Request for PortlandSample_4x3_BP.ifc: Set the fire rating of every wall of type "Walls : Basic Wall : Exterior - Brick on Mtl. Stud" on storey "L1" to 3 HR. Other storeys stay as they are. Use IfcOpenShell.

First a look at what the model holds.

```python
import ifcopenshell
import ifcopenshell.util.element

model = ifcopenshell.open("PortlandSample_4x3_BP.ifc")
print(model.schema)
storey = next(s for s in model.by_type("IfcBuildingStorey") if s.Name == "L1")
walls = [e for e in ifcopenshell.util.element.get_decomposition(storey) if e.is_a("IfcWall")]
seen = {}
for e in walls:
    element_type = ifcopenshell.util.element.get_type(e)
    key = (element_type.Name if element_type != e and element_type else None, ifcopenshell.util.element.get_pset(e, "Pset_WallCommon", "FireRating"))
    seen[key] = seen.get(key, 0) + 1
for (name, value), count in sorted(seen.items(), key=str):
    print(count, "x", name, "|", value)
```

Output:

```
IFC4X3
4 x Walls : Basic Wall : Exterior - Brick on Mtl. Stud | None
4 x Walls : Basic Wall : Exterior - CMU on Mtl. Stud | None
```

```python
import ifcopenshell
import ifcopenshell.api.pset
import ifcopenshell.util.element

model = ifcopenshell.open("PortlandSample_4x3_BP.ifc")

storey = next(s for s in model.by_type("IfcBuildingStorey") if s.Name == "L1")
walls = [e for e in ifcopenshell.util.element.get_decomposition(storey) if e.is_a("IfcWall")]

count = 0
for e in walls:
    element_type = ifcopenshell.util.element.get_type(e)
    if element_type in (None, e) or element_type.Name != "Walls : Basic Wall : Exterior - Brick on Mtl. Stud":
        continue
    # add_pset returns the element's existing set when there is one.
    pset = ifcopenshell.api.pset.add_pset(model, product=e, name="Pset_WallCommon")
    ifcopenshell.api.pset.edit_pset(model, pset=pset, properties={"FireRating": "3 HR"})
    count += 1

print(count, "walls updated")

model.write("PortlandSample_4x3_BP_rev.ifc")
```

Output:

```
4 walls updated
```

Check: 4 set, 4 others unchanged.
